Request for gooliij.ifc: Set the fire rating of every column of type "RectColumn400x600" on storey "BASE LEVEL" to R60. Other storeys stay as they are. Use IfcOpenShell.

First a look at what the model holds.

```python
import ifcopenshell
import ifcopenshell.util.element

model = ifcopenshell.open("gooliij.ifc")
print(model.schema)
storey = next(s for s in model.by_type("IfcBuildingStorey") if s.Name == "BASE LEVEL")
columns = [e for e in ifcopenshell.util.element.get_decomposition(storey) if e.is_a("IfcColumn")]
seen = {}
for e in columns:
    element_type = ifcopenshell.util.element.get_type(e)
    key = (element_type.Name if element_type != e and element_type else None, ifcopenshell.util.element.get_pset(e, "Pset_ColumnCommon", "FireRating"))
    seen[key] = seen.get(key, 0) + 1
for (name, value), count in sorted(seen.items(), key=str):
    print(count, "x", name, "|", value)
```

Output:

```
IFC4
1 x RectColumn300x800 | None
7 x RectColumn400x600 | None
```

```python
import ifcopenshell
import ifcopenshell.api.pset
import ifcopenshell.util.element

model = ifcopenshell.open("gooliij.ifc")

storey = next(s for s in model.by_type("IfcBuildingStorey") if s.Name == "BASE LEVEL")
columns = [e for e in ifcopenshell.util.element.get_decomposition(storey) if e.is_a("IfcColumn")]

count = 0
for e in columns:
    element_type = ifcopenshell.util.element.get_type(e)
    if element_type in (None, e) or element_type.Name != "RectColumn400x600":
        continue
    # add_pset returns the element's existing set when there is one.
    pset = ifcopenshell.api.pset.add_pset(model, product=e, name="Pset_ColumnCommon")
    ifcopenshell.api.pset.edit_pset(model, pset=pset, properties={"FireRating": "R60"})
    count += 1

print(count, "columns updated")

model.write("gooliij_rev.ifc")
```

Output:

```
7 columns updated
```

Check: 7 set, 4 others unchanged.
